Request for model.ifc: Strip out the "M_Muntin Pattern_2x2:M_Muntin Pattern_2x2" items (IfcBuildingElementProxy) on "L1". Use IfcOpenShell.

First a look at what the model holds.

```python
import ifcopenshell
import ifcopenshell.util.element

model = ifcopenshell.open("model.ifc")
print(model.schema)
storey = next(s for s in model.by_type("IfcBuildingStorey") if s.Name == "L1")
proxies = [e for e in ifcopenshell.util.element.get_decomposition(storey) if e.is_a("IfcBuildingElementProxy")]
seen = {}
for e in proxies:
    element_type = ifcopenshell.util.element.get_type(e)
    name = element_type.Name if element_type not in (None, e) else None
    seen[name] = seen.get(name, 0) + 1
for name, count in sorted(seen.items(), key=str):
    print(count, "x", name)
```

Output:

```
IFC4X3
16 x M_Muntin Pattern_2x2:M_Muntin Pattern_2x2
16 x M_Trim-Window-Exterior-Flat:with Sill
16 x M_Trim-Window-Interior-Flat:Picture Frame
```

```python
import ifcopenshell
import ifcopenshell.api.root
import ifcopenshell.util.element

model = ifcopenshell.open("model.ifc")

storey = next(s for s in model.by_type("IfcBuildingStorey") if s.Name == "L1")
proxies = [e for e in ifcopenshell.util.element.get_decomposition(storey) if e.is_a("IfcBuildingElementProxy")]
targets = [e for e in proxies if (t := ifcopenshell.util.element.get_type(e)) not in (None, e) and t.Name == "M_Muntin Pattern_2x2:M_Muntin Pattern_2x2"]

for e in targets:
    ifcopenshell.api.root.remove_product(model, product=e)
print(len(targets), "removed")

model.write("model_updated.ifc")
```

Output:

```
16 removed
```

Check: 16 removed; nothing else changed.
